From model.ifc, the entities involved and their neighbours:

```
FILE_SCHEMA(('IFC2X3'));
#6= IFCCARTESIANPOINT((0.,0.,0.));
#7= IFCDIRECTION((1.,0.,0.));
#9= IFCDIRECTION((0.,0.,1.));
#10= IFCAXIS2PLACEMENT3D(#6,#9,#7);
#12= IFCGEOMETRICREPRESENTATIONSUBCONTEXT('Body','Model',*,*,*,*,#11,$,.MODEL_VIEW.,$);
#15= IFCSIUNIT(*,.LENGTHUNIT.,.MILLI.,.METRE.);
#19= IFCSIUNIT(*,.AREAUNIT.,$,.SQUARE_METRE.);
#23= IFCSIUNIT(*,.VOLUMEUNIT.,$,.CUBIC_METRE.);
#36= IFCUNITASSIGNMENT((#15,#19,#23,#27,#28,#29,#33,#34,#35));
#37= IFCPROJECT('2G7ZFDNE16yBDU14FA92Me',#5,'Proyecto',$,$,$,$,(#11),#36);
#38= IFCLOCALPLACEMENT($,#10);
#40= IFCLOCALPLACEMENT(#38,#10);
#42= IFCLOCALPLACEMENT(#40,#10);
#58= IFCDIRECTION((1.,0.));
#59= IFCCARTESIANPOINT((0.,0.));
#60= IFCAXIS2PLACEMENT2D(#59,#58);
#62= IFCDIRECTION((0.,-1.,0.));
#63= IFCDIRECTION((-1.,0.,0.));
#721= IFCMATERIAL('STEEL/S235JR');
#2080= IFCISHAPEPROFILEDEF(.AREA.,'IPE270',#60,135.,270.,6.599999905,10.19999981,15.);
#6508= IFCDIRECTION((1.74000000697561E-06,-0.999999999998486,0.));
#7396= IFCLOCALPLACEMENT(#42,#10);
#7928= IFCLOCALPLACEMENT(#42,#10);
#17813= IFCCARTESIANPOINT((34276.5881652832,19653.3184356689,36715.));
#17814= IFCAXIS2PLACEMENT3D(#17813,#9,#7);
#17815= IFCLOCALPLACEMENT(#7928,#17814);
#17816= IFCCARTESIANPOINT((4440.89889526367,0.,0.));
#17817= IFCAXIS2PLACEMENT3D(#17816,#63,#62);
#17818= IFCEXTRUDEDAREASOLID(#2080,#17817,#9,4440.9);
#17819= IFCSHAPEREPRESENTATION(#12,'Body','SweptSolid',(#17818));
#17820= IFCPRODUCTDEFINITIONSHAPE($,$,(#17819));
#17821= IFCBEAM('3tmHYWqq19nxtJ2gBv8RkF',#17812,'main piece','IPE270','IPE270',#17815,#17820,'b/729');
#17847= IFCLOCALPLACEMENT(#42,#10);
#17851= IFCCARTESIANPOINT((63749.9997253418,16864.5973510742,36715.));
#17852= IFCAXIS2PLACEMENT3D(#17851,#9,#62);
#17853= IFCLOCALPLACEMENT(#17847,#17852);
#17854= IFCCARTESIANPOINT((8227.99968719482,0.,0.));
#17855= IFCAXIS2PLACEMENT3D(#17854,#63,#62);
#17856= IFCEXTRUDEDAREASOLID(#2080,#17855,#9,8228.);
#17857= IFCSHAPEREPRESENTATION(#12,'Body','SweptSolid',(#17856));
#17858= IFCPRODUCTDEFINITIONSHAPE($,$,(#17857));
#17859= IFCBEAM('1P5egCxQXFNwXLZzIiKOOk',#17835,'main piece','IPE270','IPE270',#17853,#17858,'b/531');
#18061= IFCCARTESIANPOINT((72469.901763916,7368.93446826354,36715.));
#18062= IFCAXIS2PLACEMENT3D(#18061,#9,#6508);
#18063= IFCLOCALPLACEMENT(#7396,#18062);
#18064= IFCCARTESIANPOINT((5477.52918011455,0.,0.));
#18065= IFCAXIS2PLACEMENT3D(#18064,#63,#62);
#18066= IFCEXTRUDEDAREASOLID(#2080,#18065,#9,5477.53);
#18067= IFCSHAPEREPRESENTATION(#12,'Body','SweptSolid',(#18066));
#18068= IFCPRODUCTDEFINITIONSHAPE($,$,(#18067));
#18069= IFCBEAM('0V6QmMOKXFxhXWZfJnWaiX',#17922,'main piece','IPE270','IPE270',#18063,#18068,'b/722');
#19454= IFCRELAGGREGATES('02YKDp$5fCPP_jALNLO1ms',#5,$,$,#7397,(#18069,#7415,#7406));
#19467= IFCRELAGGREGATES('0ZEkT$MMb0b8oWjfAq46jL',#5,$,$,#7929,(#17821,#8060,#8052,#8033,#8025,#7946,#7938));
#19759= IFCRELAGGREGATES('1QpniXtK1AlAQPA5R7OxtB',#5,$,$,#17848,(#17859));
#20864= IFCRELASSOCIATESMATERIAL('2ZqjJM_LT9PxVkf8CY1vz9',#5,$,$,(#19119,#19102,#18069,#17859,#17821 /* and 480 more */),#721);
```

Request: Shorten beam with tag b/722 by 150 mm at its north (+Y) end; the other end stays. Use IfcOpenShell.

```python
import ifcopenshell
import ifcopenshell.util.representation

model = ifcopenshell.open("model.ifc")

member = model.by_guid("0V6QmMOKXFxhXWZfJnWaiX")
change = -150.0

# The extrusion runs towards the end named, so only its depth changes.
body = ifcopenshell.util.representation.get_representation(member, "Model", "Body")
solid = body.Items[0]
old_length = solid.Depth
solid.Depth += change

print(f"length {old_length:g} -> {solid.Depth:g}")

model.write("model-out.ifc")
```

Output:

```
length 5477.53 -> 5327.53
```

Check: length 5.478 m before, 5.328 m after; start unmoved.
